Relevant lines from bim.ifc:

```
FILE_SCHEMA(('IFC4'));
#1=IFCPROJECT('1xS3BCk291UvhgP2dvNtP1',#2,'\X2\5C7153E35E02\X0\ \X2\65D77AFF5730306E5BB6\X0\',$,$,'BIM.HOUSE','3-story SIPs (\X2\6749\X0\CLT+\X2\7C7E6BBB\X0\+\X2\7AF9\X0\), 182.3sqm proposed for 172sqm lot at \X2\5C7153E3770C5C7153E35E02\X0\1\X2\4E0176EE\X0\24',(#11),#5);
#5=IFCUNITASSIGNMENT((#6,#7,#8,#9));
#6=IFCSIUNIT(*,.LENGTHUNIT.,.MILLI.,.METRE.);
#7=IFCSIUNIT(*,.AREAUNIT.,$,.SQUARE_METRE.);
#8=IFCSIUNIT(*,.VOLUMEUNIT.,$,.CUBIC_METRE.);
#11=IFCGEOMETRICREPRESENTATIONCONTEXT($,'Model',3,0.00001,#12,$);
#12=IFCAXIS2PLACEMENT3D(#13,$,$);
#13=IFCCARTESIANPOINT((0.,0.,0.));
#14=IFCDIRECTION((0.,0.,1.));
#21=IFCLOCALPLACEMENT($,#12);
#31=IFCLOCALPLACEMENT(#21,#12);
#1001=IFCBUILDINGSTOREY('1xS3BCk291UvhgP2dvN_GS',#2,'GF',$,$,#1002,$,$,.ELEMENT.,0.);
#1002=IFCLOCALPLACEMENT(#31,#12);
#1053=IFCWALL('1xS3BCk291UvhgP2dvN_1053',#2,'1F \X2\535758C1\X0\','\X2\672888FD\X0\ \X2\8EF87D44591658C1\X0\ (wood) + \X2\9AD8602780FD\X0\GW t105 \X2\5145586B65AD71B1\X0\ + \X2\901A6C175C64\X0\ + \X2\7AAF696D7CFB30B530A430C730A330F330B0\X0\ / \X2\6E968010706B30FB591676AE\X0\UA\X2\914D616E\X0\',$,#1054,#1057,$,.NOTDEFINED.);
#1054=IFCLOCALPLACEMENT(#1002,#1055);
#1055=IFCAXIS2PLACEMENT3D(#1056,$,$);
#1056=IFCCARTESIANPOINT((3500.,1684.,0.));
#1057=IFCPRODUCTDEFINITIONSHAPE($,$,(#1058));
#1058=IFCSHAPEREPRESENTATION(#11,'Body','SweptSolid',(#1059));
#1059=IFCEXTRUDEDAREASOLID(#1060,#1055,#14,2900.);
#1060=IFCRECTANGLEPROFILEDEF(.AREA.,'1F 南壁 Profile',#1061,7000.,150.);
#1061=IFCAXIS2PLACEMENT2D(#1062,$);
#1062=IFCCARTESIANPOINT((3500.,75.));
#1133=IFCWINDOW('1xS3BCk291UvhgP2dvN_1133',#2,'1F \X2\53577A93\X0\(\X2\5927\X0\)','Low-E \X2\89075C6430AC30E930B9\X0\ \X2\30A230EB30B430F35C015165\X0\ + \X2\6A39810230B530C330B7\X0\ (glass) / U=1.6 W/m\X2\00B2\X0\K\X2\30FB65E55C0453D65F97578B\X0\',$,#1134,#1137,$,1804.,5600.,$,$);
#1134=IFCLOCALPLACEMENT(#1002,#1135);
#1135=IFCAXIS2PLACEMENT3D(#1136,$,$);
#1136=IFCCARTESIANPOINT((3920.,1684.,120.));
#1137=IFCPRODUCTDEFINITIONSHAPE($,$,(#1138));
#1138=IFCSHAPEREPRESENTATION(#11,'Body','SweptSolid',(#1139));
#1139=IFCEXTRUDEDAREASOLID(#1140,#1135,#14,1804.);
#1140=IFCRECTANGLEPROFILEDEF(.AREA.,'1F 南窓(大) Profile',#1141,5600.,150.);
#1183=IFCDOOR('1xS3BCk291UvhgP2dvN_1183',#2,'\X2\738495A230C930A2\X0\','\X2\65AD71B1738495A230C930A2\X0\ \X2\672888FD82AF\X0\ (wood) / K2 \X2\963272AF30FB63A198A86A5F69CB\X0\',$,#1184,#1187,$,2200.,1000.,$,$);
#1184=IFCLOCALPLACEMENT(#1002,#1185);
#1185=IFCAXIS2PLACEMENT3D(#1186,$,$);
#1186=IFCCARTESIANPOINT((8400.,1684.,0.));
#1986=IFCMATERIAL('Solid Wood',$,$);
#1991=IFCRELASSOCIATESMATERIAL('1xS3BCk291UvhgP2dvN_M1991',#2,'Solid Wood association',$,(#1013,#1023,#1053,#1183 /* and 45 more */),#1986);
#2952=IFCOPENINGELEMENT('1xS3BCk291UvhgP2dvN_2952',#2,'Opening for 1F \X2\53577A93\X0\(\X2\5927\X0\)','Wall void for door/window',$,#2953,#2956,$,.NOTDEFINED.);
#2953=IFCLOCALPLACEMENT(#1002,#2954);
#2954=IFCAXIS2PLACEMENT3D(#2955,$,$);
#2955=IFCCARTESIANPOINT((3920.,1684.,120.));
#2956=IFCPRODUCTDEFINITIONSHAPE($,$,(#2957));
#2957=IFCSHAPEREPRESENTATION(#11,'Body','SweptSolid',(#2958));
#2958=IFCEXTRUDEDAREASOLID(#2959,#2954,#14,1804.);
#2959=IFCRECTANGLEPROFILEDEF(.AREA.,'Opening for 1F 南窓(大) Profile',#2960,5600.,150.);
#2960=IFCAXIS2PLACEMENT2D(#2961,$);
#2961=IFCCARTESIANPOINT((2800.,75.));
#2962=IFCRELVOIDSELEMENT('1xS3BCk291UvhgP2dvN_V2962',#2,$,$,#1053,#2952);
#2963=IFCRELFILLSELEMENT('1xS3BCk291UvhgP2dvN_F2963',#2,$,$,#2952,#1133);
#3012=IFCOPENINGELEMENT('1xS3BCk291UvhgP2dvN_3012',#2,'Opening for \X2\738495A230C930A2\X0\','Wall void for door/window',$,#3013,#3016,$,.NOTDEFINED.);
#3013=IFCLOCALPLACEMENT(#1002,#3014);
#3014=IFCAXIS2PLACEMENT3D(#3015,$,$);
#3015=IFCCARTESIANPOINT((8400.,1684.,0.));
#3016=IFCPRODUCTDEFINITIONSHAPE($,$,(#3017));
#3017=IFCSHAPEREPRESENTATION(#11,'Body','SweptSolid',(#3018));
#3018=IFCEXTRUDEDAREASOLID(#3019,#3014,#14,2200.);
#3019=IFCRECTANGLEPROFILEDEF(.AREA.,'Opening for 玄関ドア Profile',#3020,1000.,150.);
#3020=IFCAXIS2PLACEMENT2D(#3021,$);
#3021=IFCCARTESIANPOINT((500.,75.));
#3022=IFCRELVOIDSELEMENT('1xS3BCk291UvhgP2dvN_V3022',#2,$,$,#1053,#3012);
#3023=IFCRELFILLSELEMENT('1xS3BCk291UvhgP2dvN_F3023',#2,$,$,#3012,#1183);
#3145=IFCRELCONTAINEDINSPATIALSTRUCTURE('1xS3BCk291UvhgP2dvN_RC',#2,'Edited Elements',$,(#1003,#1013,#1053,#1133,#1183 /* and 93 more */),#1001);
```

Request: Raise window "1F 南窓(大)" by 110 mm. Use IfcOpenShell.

```python
import numpy as np
import ifcopenshell
import ifcopenshell.api.geometry
import ifcopenshell.util.placement
import ifcopenshell.util.unit

model = ifcopenshell.open("bim.ifc")
unit_scale = ifcopenshell.util.unit.calculate_unit_scale(model)

window = model.by_guid("1xS3BCk291UvhgP2dvN_1133")
opening = window.FillsVoids[0].RelatingOpeningElement
dz = 110.0

shift = np.array([0.0, 0.0, dz])
# The window is not placed relative to its opening, so move both.
for product in (opening, window):
    matrix = ifcopenshell.util.placement.get_local_placement(product.ObjectPlacement)
    matrix[:3, 3] += shift
    ifcopenshell.api.geometry.edit_object_placement(model, product=product, matrix=matrix, is_si=False)

print(f"moved by {dz * unit_scale:+.3f} m")

model.write("bim_edited.ifc")
```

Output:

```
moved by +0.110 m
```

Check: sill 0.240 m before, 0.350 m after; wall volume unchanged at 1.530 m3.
